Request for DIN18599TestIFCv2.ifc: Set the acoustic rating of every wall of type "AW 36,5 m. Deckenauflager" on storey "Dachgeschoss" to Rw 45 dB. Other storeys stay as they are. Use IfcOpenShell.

First a look at what the model holds.

```python
import ifcopenshell
import ifcopenshell.util.element

model = ifcopenshell.open("DIN18599TestIFCv2.ifc")
print(model.schema)
storey = next(s for s in model.by_type("IfcBuildingStorey") if s.Name == "Dachgeschoss")
walls = [e for e in ifcopenshell.util.element.get_decomposition(storey) if e.is_a("IfcWall")]
seen = {}
for e in walls:
    element_type = ifcopenshell.util.element.get_type(e)
    key = (element_type.Name if element_type != e and element_type else None, ifcopenshell.util.element.get_pset(e, "Pset_WallCommon", "AcousticRating"))
    seen[key] = seen.get(key, 0) + 1
for (name, value), count in sorted(seen.items(), key=str):
    print(count, "x", name, "|", value)
```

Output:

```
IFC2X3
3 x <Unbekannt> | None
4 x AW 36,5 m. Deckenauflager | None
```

```python
import ifcopenshell
import ifcopenshell.api.pset
import ifcopenshell.util.element

model = ifcopenshell.open("DIN18599TestIFCv2.ifc")

storey = next(s for s in model.by_type("IfcBuildingStorey") if s.Name == "Dachgeschoss")
walls = [e for e in ifcopenshell.util.element.get_decomposition(storey) if e.is_a("IfcWall")]

count = 0
for e in walls:
    element_type = ifcopenshell.util.element.get_type(e)
    if element_type in (None, e) or element_type.Name != "AW 36,5 m. Deckenauflager":
        continue
    # add_pset returns the element's existing set when there is one.
    pset = ifcopenshell.api.pset.add_pset(model, product=e, name="Pset_WallCommon")
    ifcopenshell.api.pset.edit_pset(model, pset=pset, properties={"AcousticRating": "Rw 45 dB"})
    count += 1

print(count, "walls updated")

model.write("DIN18599TestIFCv2_rev.ifc")
```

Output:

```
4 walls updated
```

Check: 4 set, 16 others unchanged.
